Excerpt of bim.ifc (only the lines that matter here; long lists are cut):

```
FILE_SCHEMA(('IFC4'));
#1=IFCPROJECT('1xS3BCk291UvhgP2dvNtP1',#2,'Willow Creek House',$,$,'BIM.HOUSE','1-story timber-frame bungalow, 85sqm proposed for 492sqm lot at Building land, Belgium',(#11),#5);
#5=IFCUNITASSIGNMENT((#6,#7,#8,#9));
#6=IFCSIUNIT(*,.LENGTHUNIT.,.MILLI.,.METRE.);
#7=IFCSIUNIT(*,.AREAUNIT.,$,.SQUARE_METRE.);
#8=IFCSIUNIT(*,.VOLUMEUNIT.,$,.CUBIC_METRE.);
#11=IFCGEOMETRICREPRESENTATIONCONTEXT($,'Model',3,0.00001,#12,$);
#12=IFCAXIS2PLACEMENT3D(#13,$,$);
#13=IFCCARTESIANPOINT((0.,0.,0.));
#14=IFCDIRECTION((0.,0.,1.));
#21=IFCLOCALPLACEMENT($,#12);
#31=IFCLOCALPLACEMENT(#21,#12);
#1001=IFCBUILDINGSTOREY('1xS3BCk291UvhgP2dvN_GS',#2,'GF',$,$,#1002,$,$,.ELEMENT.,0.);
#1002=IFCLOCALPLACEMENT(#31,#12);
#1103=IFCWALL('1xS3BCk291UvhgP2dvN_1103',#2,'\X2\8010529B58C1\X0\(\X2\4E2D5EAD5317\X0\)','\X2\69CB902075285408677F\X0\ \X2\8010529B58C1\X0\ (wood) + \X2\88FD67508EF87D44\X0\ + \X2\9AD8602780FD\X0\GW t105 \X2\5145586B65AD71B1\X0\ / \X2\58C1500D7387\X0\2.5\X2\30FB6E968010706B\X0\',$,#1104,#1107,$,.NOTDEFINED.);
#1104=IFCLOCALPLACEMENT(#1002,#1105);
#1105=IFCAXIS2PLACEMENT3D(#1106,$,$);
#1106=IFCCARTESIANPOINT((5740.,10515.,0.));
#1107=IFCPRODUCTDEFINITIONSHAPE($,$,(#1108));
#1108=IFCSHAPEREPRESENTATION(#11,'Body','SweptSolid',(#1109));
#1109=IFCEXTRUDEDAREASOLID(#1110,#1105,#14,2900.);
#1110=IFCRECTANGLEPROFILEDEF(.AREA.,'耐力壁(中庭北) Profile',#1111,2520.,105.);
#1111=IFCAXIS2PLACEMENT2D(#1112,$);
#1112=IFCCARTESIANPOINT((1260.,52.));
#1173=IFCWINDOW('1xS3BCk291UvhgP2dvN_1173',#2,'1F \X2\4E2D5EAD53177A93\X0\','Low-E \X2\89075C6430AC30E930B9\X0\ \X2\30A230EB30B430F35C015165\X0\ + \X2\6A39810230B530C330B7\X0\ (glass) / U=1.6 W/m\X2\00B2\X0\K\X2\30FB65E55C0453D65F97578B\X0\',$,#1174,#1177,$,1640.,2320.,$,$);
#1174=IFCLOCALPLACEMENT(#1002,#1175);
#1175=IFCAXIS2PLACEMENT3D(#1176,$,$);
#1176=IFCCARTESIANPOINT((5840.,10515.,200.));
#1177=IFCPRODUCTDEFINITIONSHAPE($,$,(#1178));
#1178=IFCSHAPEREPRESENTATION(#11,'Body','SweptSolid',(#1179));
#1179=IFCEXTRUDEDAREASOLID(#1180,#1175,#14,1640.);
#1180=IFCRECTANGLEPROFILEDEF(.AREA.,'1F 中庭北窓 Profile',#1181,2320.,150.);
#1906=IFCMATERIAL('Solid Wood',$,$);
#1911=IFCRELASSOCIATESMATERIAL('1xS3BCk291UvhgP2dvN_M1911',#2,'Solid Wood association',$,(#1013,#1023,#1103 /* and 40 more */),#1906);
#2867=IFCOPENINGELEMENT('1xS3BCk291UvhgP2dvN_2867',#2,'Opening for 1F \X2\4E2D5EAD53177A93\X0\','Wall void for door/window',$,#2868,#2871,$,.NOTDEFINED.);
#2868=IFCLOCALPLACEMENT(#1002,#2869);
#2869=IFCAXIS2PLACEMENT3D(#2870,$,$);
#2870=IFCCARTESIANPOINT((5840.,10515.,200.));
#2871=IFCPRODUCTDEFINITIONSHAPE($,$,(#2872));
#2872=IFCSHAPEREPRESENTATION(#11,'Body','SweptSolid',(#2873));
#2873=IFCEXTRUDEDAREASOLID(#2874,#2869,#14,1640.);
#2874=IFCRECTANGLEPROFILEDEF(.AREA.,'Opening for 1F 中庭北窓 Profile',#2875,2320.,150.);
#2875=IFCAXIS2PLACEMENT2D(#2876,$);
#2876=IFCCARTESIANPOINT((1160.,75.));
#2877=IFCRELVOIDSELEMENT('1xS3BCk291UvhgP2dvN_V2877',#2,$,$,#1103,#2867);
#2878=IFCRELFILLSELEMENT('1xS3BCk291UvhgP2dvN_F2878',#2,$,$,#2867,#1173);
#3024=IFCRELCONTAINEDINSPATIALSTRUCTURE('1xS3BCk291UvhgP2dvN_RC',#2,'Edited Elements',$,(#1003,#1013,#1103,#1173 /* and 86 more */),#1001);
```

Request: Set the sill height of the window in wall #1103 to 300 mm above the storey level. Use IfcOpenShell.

```python
import numpy as np
import ifcopenshell
import ifcopenshell.api.geometry
import ifcopenshell.geom
import ifcopenshell.util.element
import ifcopenshell.util.placement
import ifcopenshell.util.shape
import ifcopenshell.util.unit

model = ifcopenshell.open("bim.ifc")
unit_scale = ifcopenshell.util.unit.calculate_unit_scale(model)

window = model.by_guid("1xS3BCk291UvhgP2dvN_1173")
opening = window.FillsVoids[0].RelatingOpeningElement
storey = ifcopenshell.util.element.get_container(window, ifc_class="IfcBuildingStorey")
level = ifcopenshell.util.placement.get_local_placement(storey.ObjectPlacement)[2, 3]

# The opening's origin need not be at the sill, so measure its lowest point.
shape = ifcopenshell.geom.create_shape(ifcopenshell.geom.settings(), opening)
bottom = ifcopenshell.util.shape.get_shape_bottom_elevation(shape, shape.geometry) / unit_scale
dz = level + 0.3 / unit_scale - bottom

shift = np.array([0.0, 0.0, dz])
# The window is not placed relative to its opening, so move both.
for product in (opening, window):
    matrix = ifcopenshell.util.placement.get_local_placement(product.ObjectPlacement)
    matrix[:3, 3] += shift
    ifcopenshell.api.geometry.edit_object_placement(model, product=product, matrix=matrix, is_si=False)

print(f"moved by {dz * unit_scale:+.3f} m")

model.write("bim-out.ifc")
```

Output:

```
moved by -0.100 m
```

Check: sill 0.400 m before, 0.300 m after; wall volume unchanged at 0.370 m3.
